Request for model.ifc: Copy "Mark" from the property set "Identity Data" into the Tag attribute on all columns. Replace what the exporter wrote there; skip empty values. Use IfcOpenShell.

First a look at what the model holds.

```python
import ifcopenshell
import ifcopenshell.util.element

model = ifcopenshell.open("model.ifc")
print(model.schema)
columns = model.by_type("IfcColumn")
print(len(columns), "columns")
for e in columns[:8]:
    source = ifcopenshell.util.element.get_pset(e, "Identity Data", "Mark")
    target = e.Tag
    print(e.id(), repr(source), repr(target), sep=" | ")
```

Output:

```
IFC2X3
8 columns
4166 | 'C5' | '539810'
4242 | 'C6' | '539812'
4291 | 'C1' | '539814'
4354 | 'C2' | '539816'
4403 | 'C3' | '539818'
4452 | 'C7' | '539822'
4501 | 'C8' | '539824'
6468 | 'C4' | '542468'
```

```python
import ifcopenshell
import ifcopenshell.util.element

model = ifcopenshell.open("model.ifc")

count = 0
for e in model.by_type("IfcColumn"):
    value = ifcopenshell.util.element.get_pset(e, "Identity Data", "Mark")
    current = e.Tag
    if not value or not value.strip() or current == value:
        continue
    e.Tag = value
    count += 1

print(count, "columns updated")

model.write("model-out.ifc")
```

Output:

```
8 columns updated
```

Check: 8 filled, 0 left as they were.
